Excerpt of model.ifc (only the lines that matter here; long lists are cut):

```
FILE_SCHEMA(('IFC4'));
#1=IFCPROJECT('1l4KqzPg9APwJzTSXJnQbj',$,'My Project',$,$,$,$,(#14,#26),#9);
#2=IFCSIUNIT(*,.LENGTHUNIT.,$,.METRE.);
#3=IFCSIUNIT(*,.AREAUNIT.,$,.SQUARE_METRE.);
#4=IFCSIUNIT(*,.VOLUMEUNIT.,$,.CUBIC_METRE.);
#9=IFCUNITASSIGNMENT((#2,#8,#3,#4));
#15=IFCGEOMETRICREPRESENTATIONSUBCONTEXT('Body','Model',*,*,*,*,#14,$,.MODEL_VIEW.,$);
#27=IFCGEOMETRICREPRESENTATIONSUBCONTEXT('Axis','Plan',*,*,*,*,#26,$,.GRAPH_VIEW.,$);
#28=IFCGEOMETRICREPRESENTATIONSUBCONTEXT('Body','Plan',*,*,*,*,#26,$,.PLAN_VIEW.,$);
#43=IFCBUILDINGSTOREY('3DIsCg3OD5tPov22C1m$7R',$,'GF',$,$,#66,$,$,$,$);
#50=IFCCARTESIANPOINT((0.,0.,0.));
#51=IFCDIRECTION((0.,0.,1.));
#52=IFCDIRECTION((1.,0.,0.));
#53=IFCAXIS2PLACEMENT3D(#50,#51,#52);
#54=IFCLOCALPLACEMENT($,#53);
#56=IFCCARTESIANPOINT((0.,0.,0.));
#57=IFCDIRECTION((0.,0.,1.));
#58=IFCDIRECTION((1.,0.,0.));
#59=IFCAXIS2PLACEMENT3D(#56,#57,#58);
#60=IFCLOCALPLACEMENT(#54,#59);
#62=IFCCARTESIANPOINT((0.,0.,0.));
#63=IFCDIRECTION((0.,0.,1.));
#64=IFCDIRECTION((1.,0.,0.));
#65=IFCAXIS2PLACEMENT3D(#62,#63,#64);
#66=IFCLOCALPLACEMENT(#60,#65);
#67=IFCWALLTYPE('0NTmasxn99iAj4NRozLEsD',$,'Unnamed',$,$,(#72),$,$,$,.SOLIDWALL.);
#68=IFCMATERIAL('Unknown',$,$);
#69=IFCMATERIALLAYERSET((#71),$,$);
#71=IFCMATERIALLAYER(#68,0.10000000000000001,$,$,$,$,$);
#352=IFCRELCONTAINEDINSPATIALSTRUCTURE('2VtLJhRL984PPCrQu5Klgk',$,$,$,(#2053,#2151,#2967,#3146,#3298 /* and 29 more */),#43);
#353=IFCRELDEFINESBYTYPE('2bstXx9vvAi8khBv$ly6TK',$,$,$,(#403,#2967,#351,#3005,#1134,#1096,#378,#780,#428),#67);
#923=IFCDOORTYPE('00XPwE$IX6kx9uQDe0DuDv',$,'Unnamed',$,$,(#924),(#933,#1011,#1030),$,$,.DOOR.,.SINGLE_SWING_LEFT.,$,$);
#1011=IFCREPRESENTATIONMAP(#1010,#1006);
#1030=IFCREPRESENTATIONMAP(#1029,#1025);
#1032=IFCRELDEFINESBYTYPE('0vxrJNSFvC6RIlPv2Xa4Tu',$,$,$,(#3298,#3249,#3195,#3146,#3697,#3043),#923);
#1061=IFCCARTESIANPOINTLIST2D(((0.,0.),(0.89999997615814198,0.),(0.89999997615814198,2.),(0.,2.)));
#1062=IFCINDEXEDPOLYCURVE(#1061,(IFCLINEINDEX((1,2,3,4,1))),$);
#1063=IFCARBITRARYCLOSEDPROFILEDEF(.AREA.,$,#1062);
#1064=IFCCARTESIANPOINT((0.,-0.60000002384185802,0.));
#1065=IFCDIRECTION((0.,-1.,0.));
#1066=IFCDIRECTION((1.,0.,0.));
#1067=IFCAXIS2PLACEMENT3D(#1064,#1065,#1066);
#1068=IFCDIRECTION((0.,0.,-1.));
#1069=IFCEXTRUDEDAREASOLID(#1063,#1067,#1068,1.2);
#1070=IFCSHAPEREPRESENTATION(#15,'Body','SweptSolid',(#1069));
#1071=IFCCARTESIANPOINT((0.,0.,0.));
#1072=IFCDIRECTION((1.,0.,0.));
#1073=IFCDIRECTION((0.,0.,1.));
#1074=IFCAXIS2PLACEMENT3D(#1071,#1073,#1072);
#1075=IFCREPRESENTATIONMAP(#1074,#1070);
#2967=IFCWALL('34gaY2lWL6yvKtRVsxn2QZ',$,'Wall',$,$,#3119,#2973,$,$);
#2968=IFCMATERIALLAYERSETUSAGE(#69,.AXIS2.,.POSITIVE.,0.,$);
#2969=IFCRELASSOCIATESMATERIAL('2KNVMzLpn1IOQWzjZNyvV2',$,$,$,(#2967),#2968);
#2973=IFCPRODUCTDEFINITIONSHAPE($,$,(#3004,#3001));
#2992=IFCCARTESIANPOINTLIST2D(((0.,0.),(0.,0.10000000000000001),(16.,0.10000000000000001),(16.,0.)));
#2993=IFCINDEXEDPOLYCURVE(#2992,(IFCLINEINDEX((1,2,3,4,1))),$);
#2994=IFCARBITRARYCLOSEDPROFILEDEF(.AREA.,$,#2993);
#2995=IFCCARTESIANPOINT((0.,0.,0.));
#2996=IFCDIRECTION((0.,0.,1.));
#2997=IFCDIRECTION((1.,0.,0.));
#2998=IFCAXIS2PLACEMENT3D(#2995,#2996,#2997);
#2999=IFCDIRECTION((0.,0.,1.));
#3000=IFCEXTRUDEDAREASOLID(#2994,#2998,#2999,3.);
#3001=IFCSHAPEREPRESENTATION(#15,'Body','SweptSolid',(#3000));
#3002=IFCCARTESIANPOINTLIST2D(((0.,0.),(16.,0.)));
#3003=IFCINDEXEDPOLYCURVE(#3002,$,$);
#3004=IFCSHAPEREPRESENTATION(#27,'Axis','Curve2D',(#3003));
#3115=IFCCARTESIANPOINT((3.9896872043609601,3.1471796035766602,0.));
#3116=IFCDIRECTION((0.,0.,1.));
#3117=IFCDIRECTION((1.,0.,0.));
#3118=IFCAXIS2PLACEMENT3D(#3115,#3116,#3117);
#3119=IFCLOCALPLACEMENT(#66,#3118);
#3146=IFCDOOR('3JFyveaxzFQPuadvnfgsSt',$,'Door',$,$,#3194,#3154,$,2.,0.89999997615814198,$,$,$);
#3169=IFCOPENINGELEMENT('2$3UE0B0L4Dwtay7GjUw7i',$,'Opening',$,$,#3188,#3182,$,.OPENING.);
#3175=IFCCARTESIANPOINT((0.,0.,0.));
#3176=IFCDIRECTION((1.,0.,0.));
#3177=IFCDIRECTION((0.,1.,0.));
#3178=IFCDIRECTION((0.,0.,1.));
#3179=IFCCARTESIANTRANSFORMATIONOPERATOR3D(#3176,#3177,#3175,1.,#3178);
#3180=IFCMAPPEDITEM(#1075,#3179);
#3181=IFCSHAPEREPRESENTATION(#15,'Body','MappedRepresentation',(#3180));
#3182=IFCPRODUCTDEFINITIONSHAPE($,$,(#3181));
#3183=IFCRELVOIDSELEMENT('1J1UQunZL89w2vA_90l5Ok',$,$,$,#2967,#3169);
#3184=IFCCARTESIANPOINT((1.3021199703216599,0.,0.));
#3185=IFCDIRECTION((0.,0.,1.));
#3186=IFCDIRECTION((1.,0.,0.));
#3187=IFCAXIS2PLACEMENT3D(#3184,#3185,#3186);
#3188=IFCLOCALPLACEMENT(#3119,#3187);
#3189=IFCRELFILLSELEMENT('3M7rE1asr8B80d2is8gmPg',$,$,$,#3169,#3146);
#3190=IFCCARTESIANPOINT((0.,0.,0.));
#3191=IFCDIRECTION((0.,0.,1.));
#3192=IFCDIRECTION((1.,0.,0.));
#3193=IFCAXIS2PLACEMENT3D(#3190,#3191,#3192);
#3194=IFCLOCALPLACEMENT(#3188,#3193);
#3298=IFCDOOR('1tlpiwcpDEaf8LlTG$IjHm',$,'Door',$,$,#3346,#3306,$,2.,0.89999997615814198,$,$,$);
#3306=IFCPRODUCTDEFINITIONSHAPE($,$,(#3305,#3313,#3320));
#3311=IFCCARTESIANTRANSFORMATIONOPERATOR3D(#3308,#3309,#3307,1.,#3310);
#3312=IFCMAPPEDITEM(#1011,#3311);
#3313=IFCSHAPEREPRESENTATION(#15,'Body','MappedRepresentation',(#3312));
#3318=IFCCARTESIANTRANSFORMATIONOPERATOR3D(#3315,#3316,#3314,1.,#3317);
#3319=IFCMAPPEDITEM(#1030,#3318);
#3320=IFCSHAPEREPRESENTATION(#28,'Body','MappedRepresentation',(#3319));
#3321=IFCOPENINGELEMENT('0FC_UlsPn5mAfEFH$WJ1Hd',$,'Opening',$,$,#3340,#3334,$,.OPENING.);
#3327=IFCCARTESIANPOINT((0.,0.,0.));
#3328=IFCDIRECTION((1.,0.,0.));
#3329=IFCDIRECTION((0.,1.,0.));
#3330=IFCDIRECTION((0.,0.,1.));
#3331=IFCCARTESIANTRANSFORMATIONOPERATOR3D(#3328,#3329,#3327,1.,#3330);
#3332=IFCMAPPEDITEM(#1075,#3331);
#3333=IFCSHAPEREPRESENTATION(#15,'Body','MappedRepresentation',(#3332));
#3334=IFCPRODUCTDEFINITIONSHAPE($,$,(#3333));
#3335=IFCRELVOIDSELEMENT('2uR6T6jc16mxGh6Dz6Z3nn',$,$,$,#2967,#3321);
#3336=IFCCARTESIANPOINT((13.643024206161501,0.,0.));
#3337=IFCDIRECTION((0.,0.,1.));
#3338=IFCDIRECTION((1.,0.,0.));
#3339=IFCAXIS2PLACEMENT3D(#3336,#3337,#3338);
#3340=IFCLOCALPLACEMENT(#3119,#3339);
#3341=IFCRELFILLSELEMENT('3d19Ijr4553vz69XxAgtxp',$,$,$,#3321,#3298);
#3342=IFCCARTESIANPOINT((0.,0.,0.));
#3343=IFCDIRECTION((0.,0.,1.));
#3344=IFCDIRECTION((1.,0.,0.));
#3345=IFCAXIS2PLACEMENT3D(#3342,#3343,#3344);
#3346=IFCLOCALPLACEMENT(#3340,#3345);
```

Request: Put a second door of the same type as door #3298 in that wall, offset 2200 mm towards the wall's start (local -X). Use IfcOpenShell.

```python
import ifcopenshell
import ifcopenshell.api.feature
import ifcopenshell.api.geometry
import ifcopenshell.api.root
import ifcopenshell.geom
import ifcopenshell.util.element
import ifcopenshell.util.placement
import ifcopenshell.util.shape
import ifcopenshell.util.unit

model = ifcopenshell.open("model.ifc")
unit_scale = ifcopenshell.util.unit.calculate_unit_scale(model)
settings = ifcopenshell.geom.settings()


def volume(element):
    """Net volume in cubic metres, openings subtracted."""
    shape = ifcopenshell.geom.create_shape(settings, element)
    return ifcopenshell.util.shape.get_volume(shape.geometry)


door = model.by_id(3298)
opening = door.FillsVoids[0].RelatingOpeningElement
wall = opening.VoidsElements[0].RelatingBuildingElement
before = volume(wall)
shift = ifcopenshell.util.placement.get_local_placement(wall.ObjectPlacement)[:3, 0] * -2.2 / unit_scale

# copy_class copies the void relationship, type, container and properties, but no geometry.
new_opening = ifcopenshell.api.root.copy_class(model, product=opening)
new_opening.Representation = ifcopenshell.util.element.copy_deep(
    model, opening.Representation, exclude=["IfcGeometricRepresentationContext", "IfcRepresentationMap"]
)
new_door = ifcopenshell.api.root.copy_class(model, product=door)
new_door.Representation = ifcopenshell.util.element.copy_deep(
    model, door.Representation, exclude=["IfcGeometricRepresentationContext", "IfcRepresentationMap"]
)
ifcopenshell.api.feature.add_filling(model, opening=new_opening, element=new_door)

for old, new in ((opening, new_opening), (door, new_door)):
    matrix = ifcopenshell.util.placement.get_local_placement(old.ObjectPlacement)
    matrix[:3, 3] += shift
    ifcopenshell.api.geometry.edit_object_placement(model, product=new, matrix=matrix, is_si=False)

after = volume(wall)

print(f"wall volume {before:.3f} -> {after:.3f} m3")

model.write("model-out.ifc")
```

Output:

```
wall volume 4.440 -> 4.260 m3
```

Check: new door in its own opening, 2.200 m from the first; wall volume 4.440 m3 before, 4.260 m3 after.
